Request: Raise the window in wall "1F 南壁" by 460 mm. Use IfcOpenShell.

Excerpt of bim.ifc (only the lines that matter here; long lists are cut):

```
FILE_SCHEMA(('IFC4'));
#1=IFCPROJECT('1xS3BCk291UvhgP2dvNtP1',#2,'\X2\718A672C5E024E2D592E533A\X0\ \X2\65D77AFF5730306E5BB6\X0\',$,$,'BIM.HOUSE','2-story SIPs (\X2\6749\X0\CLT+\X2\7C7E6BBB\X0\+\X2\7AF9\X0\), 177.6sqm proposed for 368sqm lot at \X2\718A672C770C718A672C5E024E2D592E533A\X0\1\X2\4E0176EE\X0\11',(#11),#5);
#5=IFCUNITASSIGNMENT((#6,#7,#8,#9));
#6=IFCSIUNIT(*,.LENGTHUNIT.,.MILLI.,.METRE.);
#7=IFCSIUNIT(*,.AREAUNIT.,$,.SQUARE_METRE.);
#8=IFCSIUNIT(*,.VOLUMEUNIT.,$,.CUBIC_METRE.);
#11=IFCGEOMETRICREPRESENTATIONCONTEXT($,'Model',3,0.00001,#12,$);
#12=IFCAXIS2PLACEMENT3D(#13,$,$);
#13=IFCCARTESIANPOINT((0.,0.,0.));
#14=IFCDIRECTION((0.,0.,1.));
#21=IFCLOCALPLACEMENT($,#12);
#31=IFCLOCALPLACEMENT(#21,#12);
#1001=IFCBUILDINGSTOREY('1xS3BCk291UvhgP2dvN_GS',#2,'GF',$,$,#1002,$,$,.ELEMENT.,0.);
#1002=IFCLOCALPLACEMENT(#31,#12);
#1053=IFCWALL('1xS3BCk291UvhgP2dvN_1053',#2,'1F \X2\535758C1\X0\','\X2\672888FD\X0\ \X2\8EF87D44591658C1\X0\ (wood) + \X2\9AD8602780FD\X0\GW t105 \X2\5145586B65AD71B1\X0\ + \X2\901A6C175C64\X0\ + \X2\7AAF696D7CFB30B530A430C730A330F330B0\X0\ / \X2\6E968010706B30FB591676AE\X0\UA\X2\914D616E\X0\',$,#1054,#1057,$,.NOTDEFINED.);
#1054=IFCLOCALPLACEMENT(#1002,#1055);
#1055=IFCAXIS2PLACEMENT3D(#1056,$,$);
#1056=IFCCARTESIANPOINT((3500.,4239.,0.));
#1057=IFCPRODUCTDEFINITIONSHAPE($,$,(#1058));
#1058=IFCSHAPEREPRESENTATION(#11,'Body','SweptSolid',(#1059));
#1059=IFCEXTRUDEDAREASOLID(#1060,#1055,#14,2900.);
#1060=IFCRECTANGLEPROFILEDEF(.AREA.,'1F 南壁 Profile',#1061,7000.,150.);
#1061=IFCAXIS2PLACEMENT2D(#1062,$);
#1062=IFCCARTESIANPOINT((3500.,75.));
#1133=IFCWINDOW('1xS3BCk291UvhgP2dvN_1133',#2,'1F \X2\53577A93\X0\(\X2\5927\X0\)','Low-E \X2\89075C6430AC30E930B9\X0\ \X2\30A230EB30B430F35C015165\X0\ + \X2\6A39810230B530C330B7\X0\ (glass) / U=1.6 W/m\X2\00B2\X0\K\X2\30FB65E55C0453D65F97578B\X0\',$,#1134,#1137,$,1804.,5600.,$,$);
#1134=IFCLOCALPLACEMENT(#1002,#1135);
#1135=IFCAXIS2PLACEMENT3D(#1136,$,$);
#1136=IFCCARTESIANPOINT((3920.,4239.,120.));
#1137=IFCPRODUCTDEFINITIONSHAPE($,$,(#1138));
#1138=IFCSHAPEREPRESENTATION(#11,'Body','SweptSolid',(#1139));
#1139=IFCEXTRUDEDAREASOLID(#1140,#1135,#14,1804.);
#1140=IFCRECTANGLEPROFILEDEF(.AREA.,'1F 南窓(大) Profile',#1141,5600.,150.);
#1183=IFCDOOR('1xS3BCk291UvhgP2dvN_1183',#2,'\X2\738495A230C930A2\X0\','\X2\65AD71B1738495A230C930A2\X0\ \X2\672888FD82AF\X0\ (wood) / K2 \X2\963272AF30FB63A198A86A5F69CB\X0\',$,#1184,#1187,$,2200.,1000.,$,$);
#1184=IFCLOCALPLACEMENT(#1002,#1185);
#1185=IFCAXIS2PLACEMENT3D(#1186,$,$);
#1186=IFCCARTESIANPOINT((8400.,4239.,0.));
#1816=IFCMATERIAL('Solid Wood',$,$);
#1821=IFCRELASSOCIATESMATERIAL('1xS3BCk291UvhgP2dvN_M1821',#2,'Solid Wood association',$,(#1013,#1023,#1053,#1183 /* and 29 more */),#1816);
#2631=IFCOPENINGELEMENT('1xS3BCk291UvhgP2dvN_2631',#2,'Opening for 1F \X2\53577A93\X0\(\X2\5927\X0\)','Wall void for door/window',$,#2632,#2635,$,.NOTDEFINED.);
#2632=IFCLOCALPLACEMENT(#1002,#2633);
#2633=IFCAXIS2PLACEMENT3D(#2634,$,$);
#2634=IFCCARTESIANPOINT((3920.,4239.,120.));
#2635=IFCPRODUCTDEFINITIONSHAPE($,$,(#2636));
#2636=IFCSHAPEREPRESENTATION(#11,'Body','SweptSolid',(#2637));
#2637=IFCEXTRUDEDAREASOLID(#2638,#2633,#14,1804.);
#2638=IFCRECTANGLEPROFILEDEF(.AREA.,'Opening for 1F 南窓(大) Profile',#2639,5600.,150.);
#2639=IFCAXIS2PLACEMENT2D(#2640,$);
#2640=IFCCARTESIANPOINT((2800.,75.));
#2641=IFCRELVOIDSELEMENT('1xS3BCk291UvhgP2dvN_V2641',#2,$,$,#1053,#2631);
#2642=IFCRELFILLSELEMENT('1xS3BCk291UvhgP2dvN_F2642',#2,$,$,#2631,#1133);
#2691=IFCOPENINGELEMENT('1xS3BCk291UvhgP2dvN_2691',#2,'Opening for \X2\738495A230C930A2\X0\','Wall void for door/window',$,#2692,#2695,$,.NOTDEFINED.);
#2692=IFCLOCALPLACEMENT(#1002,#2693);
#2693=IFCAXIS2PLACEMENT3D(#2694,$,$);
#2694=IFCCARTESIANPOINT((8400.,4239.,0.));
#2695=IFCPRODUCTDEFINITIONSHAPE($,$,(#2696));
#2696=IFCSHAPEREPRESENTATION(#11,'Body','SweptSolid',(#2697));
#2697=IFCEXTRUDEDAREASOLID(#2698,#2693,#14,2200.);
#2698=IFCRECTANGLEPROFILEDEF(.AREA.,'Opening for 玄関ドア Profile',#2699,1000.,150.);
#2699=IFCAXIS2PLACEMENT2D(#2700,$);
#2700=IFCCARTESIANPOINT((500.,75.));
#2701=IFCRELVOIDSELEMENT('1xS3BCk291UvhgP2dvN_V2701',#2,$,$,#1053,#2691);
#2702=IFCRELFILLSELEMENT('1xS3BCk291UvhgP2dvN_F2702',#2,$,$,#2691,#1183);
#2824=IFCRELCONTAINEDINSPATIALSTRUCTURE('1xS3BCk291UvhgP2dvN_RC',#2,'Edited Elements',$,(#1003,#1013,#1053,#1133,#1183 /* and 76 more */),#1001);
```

```python
import numpy as np
import ifcopenshell
import ifcopenshell.api.geometry
import ifcopenshell.util.placement
import ifcopenshell.util.unit

model = ifcopenshell.open("bim.ifc")
unit_scale = ifcopenshell.util.unit.calculate_unit_scale(model)

window = model.by_guid("1xS3BCk291UvhgP2dvN_1133")
opening = window.FillsVoids[0].RelatingOpeningElement
dz = 0.46 / unit_scale

shift = np.array([0.0, 0.0, dz])
# The window is not placed relative to its opening, so move both.
for product in (opening, window):
    matrix = ifcopenshell.util.placement.get_local_placement(product.ObjectPlacement)
    matrix[:3, 3] += shift
    ifcopenshell.api.geometry.edit_object_placement(model, product=product, matrix=matrix, is_si=False)

print(f"moved by {dz * unit_scale:+.3f} m")

model.write("bim_v2.ifc")
```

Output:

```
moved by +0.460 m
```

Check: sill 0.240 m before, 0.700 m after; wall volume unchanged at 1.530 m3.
